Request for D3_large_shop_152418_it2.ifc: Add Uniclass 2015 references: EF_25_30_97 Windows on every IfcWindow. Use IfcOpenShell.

First a look at what the model holds.

```python
import ifcopenshell

model = ifcopenshell.open("D3_large_shop_152418_it2.ifc")
print(model.schema)
print("classifications:", [c.Name for c in model.by_type("IfcClassification")])
for ifc_class in ("IfcDoor", "IfcRoof", "IfcStair", "IfcWall", "IfcWindow"):
    print(ifc_class, len(model.by_type(ifc_class)))
```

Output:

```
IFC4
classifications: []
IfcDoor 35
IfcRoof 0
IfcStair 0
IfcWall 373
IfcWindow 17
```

```python
import ifcopenshell
import ifcopenshell.api.classification

model = ifcopenshell.open("D3_large_shop_152418_it2.ifc")

system = ifcopenshell.api.classification.add_classification(model, classification="Uniclass 2015")

codes = {
    "IfcWindow": ("EF_25_30_97", "Windows"),
}
for ifc_class, (code, name) in codes.items():
    products = model.by_type(ifc_class)
    ifcopenshell.api.classification.add_reference(
        model, products=products, classification=system, identification=code, name=name
    )
    print(code, len(products))

model.write("D3_large_shop_152418_it2_updated.ifc")
```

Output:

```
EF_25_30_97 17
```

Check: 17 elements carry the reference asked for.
